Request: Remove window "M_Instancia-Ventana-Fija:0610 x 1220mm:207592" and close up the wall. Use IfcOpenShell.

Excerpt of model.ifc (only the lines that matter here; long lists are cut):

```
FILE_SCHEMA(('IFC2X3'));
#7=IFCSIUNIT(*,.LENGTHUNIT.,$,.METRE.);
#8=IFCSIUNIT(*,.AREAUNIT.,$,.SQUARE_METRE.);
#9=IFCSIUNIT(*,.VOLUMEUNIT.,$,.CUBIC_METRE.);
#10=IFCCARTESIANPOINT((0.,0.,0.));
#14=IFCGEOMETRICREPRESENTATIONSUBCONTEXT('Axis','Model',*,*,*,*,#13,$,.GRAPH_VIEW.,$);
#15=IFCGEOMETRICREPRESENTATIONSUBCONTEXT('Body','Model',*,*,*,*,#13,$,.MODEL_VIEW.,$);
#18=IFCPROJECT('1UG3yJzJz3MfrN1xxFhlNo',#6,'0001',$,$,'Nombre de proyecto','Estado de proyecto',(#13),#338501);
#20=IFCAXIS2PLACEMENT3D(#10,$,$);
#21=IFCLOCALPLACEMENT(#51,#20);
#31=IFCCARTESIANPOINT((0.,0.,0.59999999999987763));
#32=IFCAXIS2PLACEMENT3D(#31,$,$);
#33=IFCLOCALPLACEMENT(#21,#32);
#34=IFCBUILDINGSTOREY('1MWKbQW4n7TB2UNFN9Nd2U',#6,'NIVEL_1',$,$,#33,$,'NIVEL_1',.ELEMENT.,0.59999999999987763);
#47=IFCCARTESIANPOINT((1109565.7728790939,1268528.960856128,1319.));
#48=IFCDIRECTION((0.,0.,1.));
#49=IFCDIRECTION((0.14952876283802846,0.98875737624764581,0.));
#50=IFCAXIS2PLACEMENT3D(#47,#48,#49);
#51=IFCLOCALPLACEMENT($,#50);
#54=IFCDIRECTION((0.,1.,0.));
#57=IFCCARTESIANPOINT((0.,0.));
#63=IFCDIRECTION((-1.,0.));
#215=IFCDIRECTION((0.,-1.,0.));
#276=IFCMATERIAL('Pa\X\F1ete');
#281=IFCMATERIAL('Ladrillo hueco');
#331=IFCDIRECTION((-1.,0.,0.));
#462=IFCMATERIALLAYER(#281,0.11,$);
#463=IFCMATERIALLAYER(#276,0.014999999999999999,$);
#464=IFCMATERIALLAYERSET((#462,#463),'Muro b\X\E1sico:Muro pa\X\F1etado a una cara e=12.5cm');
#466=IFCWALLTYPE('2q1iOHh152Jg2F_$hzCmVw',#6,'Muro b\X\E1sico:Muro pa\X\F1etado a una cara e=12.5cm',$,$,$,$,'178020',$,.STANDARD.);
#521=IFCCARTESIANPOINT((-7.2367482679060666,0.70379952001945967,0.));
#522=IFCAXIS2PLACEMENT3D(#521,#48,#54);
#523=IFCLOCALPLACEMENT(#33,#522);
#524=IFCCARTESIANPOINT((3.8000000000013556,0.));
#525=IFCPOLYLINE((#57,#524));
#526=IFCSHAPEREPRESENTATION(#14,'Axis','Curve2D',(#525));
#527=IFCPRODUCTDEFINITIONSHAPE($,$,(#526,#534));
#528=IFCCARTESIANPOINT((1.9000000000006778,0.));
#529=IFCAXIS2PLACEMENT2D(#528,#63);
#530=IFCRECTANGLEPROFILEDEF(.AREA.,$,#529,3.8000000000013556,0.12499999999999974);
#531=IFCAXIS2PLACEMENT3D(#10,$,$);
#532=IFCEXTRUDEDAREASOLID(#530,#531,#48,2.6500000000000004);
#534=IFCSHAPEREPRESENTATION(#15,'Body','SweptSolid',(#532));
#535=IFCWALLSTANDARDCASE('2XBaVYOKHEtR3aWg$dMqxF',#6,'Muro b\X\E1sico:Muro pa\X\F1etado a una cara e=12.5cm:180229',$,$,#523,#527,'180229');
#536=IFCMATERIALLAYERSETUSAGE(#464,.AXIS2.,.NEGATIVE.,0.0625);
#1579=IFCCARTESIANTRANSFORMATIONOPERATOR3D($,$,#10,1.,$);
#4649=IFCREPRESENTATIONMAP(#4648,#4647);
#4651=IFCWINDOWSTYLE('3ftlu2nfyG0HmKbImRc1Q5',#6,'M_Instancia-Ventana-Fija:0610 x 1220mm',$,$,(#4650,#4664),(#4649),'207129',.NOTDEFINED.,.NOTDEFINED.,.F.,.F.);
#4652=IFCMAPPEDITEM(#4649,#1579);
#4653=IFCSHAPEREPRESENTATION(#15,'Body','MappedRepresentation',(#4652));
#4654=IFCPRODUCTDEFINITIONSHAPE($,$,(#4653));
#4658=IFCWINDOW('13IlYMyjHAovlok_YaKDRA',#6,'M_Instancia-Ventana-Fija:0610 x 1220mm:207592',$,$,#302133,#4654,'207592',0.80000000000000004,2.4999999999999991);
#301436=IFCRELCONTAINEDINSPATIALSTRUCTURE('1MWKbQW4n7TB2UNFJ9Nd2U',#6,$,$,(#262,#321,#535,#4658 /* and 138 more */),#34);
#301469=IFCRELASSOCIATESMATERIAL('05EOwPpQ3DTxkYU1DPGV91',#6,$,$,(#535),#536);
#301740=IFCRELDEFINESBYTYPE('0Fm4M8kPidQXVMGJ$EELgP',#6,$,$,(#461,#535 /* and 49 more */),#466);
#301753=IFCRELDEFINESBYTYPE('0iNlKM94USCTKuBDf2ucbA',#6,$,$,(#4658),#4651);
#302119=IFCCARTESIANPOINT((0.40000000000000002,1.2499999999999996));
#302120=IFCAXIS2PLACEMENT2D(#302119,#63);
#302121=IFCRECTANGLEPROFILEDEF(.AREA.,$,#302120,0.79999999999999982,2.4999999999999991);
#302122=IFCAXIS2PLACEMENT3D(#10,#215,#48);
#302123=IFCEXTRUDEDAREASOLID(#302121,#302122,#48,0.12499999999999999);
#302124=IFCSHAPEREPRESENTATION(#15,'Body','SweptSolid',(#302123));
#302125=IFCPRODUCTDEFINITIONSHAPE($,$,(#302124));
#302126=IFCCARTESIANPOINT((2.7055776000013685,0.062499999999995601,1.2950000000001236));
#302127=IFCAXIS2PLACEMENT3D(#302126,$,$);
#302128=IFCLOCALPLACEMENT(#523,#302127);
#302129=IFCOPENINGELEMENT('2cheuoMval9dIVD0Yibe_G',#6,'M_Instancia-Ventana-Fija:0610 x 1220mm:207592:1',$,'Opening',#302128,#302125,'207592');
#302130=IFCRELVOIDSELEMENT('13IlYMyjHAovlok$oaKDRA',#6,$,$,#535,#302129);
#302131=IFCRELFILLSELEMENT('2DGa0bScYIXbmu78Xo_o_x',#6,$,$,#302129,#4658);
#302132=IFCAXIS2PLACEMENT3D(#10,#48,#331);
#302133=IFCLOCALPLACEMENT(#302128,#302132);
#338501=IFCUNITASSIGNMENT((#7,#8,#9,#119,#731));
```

```python
import ifcopenshell
import ifcopenshell.api.feature
import ifcopenshell.api.root
import ifcopenshell.geom
import ifcopenshell.util.shape

model = ifcopenshell.open("model.ifc")
settings = ifcopenshell.geom.settings()


def volume(element):
    """Net volume in cubic metres, openings subtracted."""
    shape = ifcopenshell.geom.create_shape(settings, element)
    return ifcopenshell.util.shape.get_volume(shape.geometry)


window = model.by_id(4658)
opening = window.FillsVoids[0].RelatingOpeningElement
wall = opening.VoidsElements[0].RelatingBuildingElement
before = volume(wall)

ifcopenshell.api.root.remove_product(model, product=window)
ifcopenshell.api.feature.remove_feature(model, feature=opening)

after = volume(wall)

print(f"wall volume {before:.3f} -> {after:.3f} m3")

model.write("model_v2.ifc")
```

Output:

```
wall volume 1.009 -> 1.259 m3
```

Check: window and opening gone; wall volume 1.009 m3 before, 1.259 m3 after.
